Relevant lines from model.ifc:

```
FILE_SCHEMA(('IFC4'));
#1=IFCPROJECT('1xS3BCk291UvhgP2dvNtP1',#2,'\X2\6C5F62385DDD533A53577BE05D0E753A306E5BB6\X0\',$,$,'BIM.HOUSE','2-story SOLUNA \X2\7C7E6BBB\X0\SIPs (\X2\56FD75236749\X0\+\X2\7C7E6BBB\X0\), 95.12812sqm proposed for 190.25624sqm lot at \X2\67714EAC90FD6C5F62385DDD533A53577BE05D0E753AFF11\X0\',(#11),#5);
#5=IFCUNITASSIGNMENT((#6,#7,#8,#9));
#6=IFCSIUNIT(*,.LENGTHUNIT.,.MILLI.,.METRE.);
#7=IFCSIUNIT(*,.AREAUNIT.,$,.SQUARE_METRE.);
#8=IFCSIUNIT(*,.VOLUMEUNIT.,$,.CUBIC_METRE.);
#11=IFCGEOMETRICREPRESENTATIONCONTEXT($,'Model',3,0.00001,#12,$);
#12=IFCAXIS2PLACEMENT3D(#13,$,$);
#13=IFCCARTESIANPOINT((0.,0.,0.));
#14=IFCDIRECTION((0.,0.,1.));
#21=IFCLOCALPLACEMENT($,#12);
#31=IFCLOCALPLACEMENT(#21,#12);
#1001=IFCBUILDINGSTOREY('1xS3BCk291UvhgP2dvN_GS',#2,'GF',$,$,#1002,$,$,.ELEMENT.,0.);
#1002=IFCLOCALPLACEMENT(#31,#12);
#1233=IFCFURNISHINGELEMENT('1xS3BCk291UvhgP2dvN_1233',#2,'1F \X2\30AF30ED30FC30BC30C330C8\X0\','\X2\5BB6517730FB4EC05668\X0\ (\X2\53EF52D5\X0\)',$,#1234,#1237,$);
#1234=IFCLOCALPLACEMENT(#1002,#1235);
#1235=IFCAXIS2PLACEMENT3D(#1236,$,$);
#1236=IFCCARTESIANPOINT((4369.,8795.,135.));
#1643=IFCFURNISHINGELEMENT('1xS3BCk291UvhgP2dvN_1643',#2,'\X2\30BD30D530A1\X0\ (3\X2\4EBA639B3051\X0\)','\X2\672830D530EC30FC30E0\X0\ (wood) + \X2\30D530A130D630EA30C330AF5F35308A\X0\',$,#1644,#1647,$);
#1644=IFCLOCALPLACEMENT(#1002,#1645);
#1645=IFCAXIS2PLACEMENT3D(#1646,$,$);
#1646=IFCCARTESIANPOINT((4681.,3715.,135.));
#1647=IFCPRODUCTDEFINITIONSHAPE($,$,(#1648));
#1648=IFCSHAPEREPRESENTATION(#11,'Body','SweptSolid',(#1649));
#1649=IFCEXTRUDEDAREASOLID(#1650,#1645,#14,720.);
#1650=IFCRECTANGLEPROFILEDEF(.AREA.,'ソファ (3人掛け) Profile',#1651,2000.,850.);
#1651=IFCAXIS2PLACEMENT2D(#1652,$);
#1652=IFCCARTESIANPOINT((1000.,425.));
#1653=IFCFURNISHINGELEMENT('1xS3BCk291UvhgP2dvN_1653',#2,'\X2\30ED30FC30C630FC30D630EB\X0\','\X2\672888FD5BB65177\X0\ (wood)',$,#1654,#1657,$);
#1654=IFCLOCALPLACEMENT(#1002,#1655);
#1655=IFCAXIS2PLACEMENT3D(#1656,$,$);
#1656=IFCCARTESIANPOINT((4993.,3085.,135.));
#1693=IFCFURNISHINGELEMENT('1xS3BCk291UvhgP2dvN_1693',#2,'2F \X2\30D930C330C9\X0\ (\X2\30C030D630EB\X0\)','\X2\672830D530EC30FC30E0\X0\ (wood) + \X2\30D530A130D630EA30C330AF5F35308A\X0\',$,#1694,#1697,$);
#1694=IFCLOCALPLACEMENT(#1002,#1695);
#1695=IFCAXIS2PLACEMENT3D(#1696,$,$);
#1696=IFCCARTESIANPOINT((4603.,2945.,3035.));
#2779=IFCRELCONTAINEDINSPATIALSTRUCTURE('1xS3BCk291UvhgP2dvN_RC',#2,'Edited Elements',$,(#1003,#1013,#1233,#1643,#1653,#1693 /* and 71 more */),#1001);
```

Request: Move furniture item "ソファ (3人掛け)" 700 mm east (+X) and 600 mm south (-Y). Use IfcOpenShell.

```python
import ifcopenshell
import ifcopenshell.api.geometry
import ifcopenshell.util.placement

model = ifcopenshell.open("model.ifc")

item = model.by_guid("1xS3BCk291UvhgP2dvN_1643")
matrix = ifcopenshell.util.placement.get_local_placement(item.ObjectPlacement)
matrix[0, 3] += 700.0
matrix[1, 3] -= 600.0
ifcopenshell.api.geometry.edit_object_placement(model, product=item, matrix=matrix, is_si=False)

print(ifcopenshell.util.placement.get_local_placement(item.ObjectPlacement).round(3) + 0.0)

model.write("model_updated.ifc")
```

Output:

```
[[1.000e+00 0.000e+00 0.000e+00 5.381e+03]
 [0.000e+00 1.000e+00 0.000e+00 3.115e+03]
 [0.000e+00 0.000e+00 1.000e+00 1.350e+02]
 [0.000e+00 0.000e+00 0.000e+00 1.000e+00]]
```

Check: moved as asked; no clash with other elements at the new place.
